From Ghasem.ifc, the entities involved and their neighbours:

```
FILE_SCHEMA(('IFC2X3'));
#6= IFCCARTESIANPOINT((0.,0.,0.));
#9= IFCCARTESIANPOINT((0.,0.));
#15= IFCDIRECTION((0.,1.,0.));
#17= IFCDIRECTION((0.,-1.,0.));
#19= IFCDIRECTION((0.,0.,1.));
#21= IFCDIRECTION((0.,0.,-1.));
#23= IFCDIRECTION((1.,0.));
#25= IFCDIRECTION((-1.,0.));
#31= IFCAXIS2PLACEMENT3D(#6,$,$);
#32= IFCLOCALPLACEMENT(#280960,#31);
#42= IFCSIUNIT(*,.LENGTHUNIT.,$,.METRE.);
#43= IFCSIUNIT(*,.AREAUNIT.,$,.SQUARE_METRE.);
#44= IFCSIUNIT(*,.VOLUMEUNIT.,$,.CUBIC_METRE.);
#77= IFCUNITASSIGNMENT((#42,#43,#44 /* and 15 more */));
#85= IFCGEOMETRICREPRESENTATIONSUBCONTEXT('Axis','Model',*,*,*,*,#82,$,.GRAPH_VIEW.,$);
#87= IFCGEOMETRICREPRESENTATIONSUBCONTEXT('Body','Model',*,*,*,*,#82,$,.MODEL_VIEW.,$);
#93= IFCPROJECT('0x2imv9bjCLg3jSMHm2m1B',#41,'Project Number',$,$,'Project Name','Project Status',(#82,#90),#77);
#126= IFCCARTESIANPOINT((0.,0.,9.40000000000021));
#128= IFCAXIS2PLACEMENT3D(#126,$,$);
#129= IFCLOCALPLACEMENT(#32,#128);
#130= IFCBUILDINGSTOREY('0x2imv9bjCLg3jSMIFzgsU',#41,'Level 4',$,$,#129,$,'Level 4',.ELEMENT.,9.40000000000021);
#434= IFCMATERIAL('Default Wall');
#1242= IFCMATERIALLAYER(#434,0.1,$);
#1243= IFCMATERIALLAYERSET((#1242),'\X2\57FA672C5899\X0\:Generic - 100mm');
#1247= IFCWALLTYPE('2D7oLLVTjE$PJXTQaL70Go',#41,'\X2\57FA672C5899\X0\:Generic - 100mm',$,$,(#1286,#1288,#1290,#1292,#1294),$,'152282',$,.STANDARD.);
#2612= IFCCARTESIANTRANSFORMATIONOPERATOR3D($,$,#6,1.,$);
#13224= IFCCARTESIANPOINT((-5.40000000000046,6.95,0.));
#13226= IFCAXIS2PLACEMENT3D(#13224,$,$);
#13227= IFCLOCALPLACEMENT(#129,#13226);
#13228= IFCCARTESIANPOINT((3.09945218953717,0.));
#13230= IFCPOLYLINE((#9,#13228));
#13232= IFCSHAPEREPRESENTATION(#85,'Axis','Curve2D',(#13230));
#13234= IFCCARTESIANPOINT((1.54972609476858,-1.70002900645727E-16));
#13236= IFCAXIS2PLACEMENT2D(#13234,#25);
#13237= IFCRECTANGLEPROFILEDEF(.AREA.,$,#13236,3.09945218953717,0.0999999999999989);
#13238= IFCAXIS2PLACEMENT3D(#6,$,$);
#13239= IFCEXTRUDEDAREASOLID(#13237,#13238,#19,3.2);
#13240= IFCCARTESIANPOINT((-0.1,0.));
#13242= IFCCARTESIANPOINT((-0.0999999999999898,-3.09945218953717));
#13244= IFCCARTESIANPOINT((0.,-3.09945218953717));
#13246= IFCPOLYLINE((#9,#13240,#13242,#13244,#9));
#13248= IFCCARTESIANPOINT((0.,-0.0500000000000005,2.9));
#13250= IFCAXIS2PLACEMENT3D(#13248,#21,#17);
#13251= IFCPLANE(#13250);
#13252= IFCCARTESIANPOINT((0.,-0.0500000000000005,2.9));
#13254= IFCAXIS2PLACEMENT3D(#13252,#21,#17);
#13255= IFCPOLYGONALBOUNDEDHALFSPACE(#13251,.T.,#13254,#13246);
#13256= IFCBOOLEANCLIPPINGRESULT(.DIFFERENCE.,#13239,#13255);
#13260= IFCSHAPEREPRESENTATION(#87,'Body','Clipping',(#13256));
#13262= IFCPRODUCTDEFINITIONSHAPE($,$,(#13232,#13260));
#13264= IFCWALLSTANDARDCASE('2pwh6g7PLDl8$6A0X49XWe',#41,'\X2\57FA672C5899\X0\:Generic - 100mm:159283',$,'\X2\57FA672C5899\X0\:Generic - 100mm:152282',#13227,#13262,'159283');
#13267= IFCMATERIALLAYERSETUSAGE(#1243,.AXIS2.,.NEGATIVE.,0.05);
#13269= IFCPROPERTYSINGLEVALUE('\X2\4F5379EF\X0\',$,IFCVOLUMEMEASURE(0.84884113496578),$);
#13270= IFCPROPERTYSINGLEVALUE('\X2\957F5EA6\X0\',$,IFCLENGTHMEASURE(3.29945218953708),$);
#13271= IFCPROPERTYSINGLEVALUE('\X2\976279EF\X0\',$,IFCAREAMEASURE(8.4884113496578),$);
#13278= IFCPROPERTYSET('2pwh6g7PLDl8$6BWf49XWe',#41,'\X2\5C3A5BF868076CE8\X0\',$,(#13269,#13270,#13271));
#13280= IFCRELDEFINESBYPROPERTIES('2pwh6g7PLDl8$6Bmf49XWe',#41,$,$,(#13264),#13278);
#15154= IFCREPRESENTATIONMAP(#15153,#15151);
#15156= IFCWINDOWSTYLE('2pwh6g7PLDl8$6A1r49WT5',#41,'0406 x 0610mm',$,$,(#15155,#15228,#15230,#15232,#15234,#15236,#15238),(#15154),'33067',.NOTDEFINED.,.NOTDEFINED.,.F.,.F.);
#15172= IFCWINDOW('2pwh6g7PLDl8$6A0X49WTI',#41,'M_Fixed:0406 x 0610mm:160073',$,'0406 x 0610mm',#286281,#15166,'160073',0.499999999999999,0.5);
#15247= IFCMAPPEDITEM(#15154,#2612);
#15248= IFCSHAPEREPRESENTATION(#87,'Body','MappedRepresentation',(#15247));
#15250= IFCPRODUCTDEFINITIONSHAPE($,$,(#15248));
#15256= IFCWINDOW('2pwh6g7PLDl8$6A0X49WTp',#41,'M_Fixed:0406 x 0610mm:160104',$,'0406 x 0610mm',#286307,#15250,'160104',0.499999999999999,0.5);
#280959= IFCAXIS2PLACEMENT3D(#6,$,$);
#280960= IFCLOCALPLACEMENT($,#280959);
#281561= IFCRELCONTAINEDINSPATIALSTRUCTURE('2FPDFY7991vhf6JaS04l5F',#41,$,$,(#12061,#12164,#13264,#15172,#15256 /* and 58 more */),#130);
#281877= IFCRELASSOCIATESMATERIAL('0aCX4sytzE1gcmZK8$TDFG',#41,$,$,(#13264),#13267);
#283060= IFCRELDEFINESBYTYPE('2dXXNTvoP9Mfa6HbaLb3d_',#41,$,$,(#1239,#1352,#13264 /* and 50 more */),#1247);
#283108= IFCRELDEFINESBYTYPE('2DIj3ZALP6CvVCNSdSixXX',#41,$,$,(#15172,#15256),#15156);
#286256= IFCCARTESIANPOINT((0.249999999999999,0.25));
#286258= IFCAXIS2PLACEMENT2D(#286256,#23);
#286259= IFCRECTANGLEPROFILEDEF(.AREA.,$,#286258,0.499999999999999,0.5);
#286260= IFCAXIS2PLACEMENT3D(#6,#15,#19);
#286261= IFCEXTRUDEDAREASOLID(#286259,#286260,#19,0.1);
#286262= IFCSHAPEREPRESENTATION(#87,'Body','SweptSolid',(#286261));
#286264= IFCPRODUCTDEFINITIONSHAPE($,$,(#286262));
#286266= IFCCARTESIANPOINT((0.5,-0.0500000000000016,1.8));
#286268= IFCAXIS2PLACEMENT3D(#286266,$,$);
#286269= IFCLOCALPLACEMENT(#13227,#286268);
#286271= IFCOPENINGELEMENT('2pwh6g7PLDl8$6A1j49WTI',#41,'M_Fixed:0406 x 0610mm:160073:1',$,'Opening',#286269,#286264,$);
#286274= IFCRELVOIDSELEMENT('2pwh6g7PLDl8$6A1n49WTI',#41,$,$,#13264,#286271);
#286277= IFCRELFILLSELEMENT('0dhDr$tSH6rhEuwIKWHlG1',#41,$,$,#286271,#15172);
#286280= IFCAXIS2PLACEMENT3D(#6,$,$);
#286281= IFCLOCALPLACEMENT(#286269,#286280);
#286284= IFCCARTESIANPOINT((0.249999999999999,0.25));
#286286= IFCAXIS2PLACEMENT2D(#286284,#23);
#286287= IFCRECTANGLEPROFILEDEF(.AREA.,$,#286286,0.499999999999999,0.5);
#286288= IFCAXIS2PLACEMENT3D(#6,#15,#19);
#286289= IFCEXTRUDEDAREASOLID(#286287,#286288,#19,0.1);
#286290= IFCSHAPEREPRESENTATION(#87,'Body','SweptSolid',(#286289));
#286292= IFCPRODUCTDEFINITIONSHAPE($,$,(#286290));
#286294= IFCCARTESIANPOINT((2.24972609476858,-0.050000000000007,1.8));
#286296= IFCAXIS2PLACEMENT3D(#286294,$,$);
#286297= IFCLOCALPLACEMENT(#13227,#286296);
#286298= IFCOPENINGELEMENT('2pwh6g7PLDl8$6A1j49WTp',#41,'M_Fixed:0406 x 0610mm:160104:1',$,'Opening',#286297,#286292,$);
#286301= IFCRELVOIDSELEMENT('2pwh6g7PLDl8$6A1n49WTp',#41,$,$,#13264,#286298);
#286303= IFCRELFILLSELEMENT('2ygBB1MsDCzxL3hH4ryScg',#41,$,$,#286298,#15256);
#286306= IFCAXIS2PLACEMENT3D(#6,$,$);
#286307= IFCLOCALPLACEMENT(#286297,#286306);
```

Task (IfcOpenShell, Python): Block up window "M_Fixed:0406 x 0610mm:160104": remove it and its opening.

```python
import ifcopenshell
import ifcopenshell.api.feature
import ifcopenshell.api.pset
import ifcopenshell.api.root
import ifcopenshell.geom
import ifcopenshell.util.element
import ifcopenshell.util.shape
import ifcopenshell.util.unit

model = ifcopenshell.open("Ghasem.ifc")
area_scale = ifcopenshell.util.unit.calculate_unit_scale(model, "AREAUNIT")
volume_scale = ifcopenshell.util.unit.calculate_unit_scale(model, "VOLUMEUNIT")
settings = ifcopenshell.geom.settings()


def volume(element):
    """Net volume in cubic metres, openings subtracted."""
    shape = ifcopenshell.geom.create_shape(settings, element)
    return ifcopenshell.util.shape.get_volume(shape.geometry)


window = model.by_guid("2pwh6g7PLDl8$6A0X49WTp")
opening = window.FillsVoids[0].RelatingOpeningElement
wall = opening.VoidsElements[0].RelatingBuildingElement
before = volume(wall)

ifcopenshell.api.root.remove_product(model, product=window)
ifcopenshell.api.feature.remove_feature(model, feature=opening)

after = volume(wall)
thickness = 0.1  # wall thickness in metres

# Update the wall's stored quantities.
pset = model.by_id(ifcopenshell.util.element.get_pset(wall, "尺寸标注", should_inherit=False)["id"])
ifcopenshell.api.pset.edit_pset(model, pset=pset, properties={
    "体积": model.create_entity("IfcVolumeMeasure", after / volume_scale),
    "面积": model.create_entity("IfcAreaMeasure", after / thickness / area_scale),
})

print(f"wall volume {before:.3f} -> {after:.3f} m3")

model.write("Ghasem-out.ifc")
```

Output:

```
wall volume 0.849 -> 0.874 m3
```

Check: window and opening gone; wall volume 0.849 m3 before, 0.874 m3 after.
